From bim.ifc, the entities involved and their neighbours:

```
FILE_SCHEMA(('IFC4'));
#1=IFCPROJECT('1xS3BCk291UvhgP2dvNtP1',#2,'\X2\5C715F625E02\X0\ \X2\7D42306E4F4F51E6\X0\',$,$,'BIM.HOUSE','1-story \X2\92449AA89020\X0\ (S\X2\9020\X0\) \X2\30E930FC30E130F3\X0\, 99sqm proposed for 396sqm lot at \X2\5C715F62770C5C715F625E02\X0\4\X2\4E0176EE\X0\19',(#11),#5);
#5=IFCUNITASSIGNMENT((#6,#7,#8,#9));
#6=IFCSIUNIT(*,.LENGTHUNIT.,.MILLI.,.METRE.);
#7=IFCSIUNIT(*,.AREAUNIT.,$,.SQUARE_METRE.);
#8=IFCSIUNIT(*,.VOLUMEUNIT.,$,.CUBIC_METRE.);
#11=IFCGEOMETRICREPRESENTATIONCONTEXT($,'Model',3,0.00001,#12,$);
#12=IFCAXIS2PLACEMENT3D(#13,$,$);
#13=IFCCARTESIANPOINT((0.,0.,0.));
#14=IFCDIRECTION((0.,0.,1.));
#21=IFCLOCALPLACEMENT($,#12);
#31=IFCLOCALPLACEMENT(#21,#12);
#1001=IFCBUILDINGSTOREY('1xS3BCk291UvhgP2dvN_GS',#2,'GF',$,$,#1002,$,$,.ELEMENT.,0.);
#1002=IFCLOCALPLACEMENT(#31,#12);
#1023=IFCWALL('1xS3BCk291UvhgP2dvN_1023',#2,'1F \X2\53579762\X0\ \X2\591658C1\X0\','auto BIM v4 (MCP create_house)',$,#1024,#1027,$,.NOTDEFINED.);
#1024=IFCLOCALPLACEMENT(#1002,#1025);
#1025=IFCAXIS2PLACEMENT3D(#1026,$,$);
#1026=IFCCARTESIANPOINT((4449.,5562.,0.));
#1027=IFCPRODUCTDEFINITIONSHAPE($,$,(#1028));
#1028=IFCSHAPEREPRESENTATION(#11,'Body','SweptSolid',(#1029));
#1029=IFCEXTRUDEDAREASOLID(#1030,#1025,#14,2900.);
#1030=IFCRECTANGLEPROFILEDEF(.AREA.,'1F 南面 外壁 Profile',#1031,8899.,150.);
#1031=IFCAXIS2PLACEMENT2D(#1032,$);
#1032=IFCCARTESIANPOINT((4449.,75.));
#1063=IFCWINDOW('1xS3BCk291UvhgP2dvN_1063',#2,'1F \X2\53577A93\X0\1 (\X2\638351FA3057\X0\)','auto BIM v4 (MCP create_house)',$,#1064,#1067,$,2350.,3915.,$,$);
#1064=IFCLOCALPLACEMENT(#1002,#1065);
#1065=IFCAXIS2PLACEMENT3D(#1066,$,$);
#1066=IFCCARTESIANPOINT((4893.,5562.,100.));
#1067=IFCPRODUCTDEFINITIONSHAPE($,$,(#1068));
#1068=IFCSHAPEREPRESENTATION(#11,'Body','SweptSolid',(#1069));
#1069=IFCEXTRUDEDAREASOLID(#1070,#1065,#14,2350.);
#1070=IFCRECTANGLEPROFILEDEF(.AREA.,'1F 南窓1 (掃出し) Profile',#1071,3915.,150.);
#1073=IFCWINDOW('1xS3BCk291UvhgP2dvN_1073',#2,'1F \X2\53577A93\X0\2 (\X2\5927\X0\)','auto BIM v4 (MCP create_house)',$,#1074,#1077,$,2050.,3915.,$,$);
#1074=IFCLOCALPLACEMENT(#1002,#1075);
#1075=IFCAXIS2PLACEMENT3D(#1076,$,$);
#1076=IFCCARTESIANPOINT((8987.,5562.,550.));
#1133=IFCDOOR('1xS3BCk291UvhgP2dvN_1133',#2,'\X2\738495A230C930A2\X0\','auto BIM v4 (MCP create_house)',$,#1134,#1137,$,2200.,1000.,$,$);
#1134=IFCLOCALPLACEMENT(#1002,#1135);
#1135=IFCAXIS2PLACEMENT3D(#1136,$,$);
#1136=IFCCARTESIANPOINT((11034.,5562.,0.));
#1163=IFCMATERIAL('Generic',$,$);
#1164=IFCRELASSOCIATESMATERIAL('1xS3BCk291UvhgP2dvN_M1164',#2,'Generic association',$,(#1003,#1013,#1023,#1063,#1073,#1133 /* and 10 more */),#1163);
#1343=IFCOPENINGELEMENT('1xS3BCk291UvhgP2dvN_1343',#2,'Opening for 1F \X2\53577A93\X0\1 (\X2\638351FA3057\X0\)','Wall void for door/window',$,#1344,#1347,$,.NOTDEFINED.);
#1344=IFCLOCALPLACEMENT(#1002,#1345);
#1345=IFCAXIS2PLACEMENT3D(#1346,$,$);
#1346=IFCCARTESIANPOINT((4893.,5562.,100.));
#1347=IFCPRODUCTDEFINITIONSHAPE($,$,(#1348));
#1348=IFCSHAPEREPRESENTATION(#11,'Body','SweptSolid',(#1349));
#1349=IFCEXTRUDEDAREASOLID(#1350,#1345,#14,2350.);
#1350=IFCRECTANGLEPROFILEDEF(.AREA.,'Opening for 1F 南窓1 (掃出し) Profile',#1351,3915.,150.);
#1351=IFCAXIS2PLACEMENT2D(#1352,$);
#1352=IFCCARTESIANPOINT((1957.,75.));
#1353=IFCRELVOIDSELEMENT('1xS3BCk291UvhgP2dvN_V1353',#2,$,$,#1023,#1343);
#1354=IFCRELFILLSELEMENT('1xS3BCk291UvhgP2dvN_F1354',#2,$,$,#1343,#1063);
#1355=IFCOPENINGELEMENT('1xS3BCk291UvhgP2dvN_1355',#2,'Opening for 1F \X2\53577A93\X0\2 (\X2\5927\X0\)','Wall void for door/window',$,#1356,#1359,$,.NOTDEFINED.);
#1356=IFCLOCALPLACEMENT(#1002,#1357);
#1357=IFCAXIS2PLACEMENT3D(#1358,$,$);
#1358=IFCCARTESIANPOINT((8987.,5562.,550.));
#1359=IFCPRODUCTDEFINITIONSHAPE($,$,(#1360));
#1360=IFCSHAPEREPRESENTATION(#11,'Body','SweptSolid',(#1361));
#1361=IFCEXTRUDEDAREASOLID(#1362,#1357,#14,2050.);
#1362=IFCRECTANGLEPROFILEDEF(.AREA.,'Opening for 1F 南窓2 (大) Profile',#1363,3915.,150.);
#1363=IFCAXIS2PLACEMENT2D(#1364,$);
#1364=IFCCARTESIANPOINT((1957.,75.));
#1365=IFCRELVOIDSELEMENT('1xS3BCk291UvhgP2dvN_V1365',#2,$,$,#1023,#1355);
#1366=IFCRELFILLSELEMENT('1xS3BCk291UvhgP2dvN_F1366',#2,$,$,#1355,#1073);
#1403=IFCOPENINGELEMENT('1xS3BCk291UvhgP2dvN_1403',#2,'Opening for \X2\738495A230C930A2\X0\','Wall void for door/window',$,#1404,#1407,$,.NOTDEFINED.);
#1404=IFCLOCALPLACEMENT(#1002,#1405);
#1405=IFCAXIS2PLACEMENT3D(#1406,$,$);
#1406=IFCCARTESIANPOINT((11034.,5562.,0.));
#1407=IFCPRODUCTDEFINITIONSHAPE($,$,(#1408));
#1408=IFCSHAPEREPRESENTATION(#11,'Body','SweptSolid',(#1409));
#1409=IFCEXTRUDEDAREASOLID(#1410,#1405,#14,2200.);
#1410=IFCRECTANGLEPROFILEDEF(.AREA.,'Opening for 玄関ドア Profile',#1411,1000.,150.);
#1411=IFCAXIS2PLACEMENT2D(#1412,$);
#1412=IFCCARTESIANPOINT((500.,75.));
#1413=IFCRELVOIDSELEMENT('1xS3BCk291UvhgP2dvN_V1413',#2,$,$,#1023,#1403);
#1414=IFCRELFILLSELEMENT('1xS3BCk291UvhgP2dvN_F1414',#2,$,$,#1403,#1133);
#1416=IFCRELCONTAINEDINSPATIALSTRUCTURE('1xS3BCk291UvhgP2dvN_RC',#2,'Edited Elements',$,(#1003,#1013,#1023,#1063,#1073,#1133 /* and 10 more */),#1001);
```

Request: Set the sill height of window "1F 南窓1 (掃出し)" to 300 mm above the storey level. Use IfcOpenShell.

```python
import numpy as np
import ifcopenshell
import ifcopenshell.api.geometry
import ifcopenshell.geom
import ifcopenshell.util.element
import ifcopenshell.util.placement
import ifcopenshell.util.shape
import ifcopenshell.util.unit

model = ifcopenshell.open("bim.ifc")
unit_scale = ifcopenshell.util.unit.calculate_unit_scale(model)

window = model.by_id(1063)
opening = window.FillsVoids[0].RelatingOpeningElement
storey = ifcopenshell.util.element.get_container(window, ifc_class="IfcBuildingStorey")
level = ifcopenshell.util.placement.get_local_placement(storey.ObjectPlacement)[2, 3]

# The opening's origin need not be at the sill, so measure its lowest point.
shape = ifcopenshell.geom.create_shape(ifcopenshell.geom.settings(), opening)
bottom = ifcopenshell.util.shape.get_shape_bottom_elevation(shape, shape.geometry) / unit_scale
dz = level + 300.0 - bottom

shift = np.array([0.0, 0.0, dz])
# The window is not placed relative to its opening, so move both.
for product in (opening, window):
    matrix = ifcopenshell.util.placement.get_local_placement(product.ObjectPlacement)
    matrix[:3, 3] += shift
    ifcopenshell.api.geometry.edit_object_placement(model, product=product, matrix=matrix, is_si=False)

print(f"moved by {dz * unit_scale:+.3f} m")

model.write("bim_updated.ifc")
```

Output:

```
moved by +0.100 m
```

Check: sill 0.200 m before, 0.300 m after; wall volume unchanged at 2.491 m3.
